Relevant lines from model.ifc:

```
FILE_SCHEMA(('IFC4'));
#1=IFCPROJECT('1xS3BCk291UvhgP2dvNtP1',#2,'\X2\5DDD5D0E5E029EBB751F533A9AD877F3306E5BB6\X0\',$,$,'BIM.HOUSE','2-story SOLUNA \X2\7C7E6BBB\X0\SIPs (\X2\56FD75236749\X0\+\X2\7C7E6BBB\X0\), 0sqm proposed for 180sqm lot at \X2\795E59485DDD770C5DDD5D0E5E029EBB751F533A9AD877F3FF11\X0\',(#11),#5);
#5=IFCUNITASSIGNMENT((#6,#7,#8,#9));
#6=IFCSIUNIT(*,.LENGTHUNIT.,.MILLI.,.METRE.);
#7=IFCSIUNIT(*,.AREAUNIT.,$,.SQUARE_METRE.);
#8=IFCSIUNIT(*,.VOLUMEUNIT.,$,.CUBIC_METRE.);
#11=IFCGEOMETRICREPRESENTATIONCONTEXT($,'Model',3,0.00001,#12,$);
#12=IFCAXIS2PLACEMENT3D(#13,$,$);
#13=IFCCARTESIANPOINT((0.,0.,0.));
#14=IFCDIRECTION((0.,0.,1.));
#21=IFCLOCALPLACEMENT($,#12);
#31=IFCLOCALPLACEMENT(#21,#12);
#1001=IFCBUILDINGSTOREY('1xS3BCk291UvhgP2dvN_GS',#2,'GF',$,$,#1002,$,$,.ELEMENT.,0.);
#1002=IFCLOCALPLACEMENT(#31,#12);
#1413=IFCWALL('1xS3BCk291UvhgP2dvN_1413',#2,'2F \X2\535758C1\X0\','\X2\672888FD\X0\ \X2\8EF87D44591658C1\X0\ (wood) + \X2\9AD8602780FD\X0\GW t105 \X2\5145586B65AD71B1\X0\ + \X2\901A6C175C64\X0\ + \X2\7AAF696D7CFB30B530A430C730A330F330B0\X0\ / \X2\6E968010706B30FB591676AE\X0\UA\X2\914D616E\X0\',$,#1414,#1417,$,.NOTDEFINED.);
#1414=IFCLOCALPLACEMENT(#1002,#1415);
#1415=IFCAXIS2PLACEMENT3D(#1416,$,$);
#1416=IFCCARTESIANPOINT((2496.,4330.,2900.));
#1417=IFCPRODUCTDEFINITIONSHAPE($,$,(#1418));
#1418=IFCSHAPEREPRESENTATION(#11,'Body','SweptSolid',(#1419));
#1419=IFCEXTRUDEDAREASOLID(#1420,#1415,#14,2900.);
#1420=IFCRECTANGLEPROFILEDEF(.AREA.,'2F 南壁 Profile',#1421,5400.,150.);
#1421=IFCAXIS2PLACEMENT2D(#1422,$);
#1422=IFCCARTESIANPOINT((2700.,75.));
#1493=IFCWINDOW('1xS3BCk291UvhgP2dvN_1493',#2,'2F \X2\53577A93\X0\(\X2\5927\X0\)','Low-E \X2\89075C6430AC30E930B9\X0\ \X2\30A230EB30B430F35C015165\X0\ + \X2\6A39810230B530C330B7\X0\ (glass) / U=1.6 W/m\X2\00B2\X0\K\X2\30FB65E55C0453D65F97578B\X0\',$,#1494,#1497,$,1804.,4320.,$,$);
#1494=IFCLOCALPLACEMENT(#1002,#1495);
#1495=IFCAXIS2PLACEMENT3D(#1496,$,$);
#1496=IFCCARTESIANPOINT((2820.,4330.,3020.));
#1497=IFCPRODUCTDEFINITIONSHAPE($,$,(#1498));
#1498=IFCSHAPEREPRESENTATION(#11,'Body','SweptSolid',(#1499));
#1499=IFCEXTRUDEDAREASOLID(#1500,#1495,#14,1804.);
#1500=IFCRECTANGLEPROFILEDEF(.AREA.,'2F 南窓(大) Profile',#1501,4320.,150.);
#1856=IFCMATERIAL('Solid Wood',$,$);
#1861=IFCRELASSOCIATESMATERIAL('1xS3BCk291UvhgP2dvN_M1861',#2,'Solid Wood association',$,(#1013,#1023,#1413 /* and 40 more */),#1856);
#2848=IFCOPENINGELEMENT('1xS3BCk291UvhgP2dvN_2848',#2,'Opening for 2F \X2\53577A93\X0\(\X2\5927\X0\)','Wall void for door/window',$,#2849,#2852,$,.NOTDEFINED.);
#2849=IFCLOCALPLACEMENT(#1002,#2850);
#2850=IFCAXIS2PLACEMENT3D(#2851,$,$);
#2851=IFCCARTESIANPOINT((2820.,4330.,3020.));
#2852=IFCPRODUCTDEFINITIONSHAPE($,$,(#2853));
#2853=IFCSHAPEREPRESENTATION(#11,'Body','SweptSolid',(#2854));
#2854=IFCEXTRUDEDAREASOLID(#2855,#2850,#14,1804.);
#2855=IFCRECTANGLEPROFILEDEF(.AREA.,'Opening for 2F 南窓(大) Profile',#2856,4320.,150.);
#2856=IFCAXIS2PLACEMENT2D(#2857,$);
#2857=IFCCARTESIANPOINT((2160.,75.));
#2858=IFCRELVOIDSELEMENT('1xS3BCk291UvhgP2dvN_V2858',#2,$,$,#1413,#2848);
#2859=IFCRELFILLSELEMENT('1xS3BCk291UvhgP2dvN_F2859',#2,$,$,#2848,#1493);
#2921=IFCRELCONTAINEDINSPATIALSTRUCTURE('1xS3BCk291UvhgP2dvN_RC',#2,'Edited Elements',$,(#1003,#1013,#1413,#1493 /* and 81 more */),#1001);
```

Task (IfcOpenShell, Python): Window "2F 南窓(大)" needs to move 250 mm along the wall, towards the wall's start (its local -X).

```python
import ifcopenshell
import ifcopenshell.api.geometry
import ifcopenshell.util.placement
import ifcopenshell.util.unit

model = ifcopenshell.open("model.ifc")
unit_scale = ifcopenshell.util.unit.calculate_unit_scale(model)

window = model.by_guid("1xS3BCk291UvhgP2dvN_1493")
opening = window.FillsVoids[0].RelatingOpeningElement
wall = opening.VoidsElements[0].RelatingBuildingElement

wall_matrix = ifcopenshell.util.placement.get_local_placement(wall.ObjectPlacement)
shift = wall_matrix[:3, 0] * -0.25 / unit_scale
before = ifcopenshell.util.placement.get_local_placement(window.ObjectPlacement)[:3, 3].copy()

# The window is not placed relative to its opening, so move both.
for product in (opening, window):
    matrix = ifcopenshell.util.placement.get_local_placement(product.ObjectPlacement)
    matrix[:3, 3] += shift
    ifcopenshell.api.geometry.edit_object_placement(model, product=product, matrix=matrix, is_si=False)

after = ifcopenshell.util.placement.get_local_placement(window.ObjectPlacement)[:3, 3]
print("window moved by", (after - before).round(3) + 0.0)

model.write("model-out.ifc")
```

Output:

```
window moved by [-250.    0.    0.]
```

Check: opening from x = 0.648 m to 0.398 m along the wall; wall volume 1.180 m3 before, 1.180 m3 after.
